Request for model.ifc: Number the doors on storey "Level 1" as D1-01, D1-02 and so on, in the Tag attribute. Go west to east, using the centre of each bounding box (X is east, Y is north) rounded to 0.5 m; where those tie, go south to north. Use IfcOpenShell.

First a look at what the model holds.

```python
import ifcopenshell
import ifcopenshell.util.element
import ifcopenshell.util.placement

model = ifcopenshell.open("model.ifc")
print(model.schema)
storey = next(s for s in model.by_type("IfcBuildingStorey") if s.Name == "Level 1")
doors = [e for e in ifcopenshell.util.element.get_decomposition(storey) if e.is_a("IfcDoor")]
for e in sorted(doors, key=lambda e: e.id()):
    origin = ifcopenshell.util.placement.get_local_placement(e.ObjectPlacement)[:3, 3]
    print(e.id(), e.Tag, e.Name, origin.round(2) + 0.0, sep=" | ")
```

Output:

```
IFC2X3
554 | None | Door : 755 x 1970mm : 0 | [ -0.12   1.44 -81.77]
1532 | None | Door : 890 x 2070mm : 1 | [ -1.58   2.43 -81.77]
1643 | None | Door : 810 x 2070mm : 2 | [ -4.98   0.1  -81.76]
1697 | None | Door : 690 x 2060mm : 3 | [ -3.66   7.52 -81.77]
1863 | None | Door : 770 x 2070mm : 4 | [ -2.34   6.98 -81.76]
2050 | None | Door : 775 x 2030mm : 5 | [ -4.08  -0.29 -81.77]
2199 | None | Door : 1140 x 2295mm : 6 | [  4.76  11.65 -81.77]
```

```python
import ifcopenshell
import ifcopenshell.geom
import ifcopenshell.util.element
import ifcopenshell.util.shape

model = ifcopenshell.open("model.ifc")
settings = ifcopenshell.geom.settings()
settings.set("use-world-coords", True)


def centre(element):
    shape = ifcopenshell.geom.create_shape(settings, element)
    return ifcopenshell.util.shape.get_bbox_centroid(shape.geometry)


storey = next(s for s in model.by_type("IfcBuildingStorey") if s.Name == "Level 1")
doors = [e for e in ifcopenshell.util.element.get_decomposition(storey) if e.is_a("IfcDoor")]

# Insertion points can sit at a corner or the storey origin, so sort by the geometry (in metres).
centres = {e: centre(e) for e in doors}
doors.sort(key=lambda e: (round(centres[e][0] / 0.5), centres[e][1]))

for i, e in enumerate(doors, start=1):
    number = f"D1-{i:02d}"
    e.Tag = number
    print(e.id(), number)

model.write("model-out.ifc")
```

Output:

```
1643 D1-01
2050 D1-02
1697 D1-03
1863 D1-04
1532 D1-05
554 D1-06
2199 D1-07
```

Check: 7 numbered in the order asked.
